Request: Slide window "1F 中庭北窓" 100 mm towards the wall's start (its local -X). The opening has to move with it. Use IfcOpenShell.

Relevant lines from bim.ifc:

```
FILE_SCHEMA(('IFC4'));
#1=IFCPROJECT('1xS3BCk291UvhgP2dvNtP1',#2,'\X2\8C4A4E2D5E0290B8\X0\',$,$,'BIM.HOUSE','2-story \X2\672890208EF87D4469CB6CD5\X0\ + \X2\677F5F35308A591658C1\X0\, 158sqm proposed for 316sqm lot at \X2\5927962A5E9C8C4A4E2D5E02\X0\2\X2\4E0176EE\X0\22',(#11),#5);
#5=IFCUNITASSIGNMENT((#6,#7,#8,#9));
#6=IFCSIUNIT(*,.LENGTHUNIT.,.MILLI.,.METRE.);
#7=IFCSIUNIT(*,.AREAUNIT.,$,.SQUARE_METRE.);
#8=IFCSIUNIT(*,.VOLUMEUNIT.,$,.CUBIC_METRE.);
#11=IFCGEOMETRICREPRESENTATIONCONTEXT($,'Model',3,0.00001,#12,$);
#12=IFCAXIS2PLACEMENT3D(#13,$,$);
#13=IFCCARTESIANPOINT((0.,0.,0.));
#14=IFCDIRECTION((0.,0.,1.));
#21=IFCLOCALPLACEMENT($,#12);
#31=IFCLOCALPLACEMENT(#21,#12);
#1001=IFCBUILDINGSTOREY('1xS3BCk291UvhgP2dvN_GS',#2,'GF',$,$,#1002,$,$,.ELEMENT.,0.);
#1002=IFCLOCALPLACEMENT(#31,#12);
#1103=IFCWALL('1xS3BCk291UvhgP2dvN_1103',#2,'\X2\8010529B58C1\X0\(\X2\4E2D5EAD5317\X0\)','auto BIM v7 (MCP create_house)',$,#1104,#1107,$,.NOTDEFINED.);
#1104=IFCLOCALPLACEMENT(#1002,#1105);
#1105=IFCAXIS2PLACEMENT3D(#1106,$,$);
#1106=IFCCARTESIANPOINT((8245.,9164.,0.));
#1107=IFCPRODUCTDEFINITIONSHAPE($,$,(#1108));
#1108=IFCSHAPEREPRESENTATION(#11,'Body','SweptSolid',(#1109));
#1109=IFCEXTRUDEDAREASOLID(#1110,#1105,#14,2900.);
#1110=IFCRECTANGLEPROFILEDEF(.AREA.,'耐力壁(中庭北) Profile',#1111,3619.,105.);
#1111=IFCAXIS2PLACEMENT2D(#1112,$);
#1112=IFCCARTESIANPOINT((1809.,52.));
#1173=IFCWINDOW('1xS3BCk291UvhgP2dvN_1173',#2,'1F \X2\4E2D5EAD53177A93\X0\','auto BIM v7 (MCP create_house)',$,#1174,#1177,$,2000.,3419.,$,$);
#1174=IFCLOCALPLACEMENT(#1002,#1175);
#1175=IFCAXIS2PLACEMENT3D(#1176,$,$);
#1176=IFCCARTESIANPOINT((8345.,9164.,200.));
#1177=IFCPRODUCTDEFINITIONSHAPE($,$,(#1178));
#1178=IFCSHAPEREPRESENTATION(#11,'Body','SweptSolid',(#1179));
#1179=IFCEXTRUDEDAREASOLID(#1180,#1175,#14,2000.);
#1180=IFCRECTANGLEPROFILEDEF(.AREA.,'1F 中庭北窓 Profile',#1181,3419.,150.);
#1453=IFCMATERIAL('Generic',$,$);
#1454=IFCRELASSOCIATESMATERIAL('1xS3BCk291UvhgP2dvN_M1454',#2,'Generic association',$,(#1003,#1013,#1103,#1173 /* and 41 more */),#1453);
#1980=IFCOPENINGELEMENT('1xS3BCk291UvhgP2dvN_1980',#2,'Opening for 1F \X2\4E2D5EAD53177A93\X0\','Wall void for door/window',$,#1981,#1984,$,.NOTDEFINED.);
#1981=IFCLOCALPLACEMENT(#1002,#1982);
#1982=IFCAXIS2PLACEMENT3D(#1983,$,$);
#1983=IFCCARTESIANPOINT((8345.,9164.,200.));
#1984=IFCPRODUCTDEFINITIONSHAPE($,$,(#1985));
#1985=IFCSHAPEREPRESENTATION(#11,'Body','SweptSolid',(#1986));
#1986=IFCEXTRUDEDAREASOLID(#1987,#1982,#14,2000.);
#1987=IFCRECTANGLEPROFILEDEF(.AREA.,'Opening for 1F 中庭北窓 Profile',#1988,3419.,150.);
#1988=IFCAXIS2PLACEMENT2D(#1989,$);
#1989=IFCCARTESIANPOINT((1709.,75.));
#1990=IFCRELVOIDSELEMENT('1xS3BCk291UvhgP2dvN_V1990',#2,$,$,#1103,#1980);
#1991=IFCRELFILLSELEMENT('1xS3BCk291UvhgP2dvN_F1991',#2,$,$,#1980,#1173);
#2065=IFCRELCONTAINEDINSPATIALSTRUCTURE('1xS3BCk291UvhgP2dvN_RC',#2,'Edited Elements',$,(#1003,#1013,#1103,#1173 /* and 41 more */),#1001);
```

```python
import ifcopenshell
import ifcopenshell.api.geometry
import ifcopenshell.util.placement

model = ifcopenshell.open("bim.ifc")

window = model.by_guid("1xS3BCk291UvhgP2dvN_1173")
opening = window.FillsVoids[0].RelatingOpeningElement
wall = opening.VoidsElements[0].RelatingBuildingElement

wall_matrix = ifcopenshell.util.placement.get_local_placement(wall.ObjectPlacement)
shift = wall_matrix[:3, 0] * -100.0
before = ifcopenshell.util.placement.get_local_placement(window.ObjectPlacement)[:3, 3].copy()

# The window is not placed relative to its opening, so move both.
for product in (opening, window):
    matrix = ifcopenshell.util.placement.get_local_placement(product.ObjectPlacement)
    matrix[:3, 3] += shift
    ifcopenshell.api.geometry.edit_object_placement(model, product=product, matrix=matrix, is_si=False)

after = ifcopenshell.util.placement.get_local_placement(window.ObjectPlacement)[:3, 3]
print("window moved by", (after - before).round(3) + 0.0)

model.write("bim_updated.ifc")
```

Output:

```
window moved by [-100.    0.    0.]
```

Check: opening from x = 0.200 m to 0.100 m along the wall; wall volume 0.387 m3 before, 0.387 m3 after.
